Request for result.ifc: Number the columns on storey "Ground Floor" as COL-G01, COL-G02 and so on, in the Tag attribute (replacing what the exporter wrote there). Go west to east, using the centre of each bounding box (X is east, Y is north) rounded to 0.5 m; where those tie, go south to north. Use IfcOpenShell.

First a look at what the model holds.

```python
import ifcopenshell
import ifcopenshell.util.element
import ifcopenshell.util.placement

model = ifcopenshell.open("result.ifc")
print(model.schema)
storey = next(s for s in model.by_type("IfcBuildingStorey") if s.Name == "Ground Floor")
columns = [e for e in ifcopenshell.util.element.get_decomposition(storey) if e.is_a("IfcColumn")]
for e in sorted(columns, key=lambda e: e.id()):
    origin = ifcopenshell.util.placement.get_local_placement(e.ObjectPlacement)[:3, 3]
    print(e.id(), e.Tag, e.Name, origin.round(2) + 0.0, sep=" | ")
```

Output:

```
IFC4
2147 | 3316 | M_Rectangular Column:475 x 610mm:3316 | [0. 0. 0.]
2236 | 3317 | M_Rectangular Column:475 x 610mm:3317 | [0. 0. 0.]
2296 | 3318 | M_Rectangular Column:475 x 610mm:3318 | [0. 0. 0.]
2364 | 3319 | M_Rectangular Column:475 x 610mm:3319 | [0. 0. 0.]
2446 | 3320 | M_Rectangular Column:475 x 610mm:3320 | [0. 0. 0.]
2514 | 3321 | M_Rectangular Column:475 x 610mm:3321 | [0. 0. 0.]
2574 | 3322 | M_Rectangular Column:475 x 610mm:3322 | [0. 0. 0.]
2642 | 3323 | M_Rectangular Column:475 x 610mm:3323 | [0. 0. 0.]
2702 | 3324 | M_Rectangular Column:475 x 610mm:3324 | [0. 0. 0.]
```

```python
import ifcopenshell
import ifcopenshell.geom
import ifcopenshell.util.element
import ifcopenshell.util.shape

model = ifcopenshell.open("result.ifc")
settings = ifcopenshell.geom.settings()
settings.set("use-world-coords", True)


def centre(element):
    shape = ifcopenshell.geom.create_shape(settings, element)
    return ifcopenshell.util.shape.get_bbox_centroid(shape.geometry)


storey = next(s for s in model.by_type("IfcBuildingStorey") if s.Name == "Ground Floor")
columns = [e for e in ifcopenshell.util.element.get_decomposition(storey) if e.is_a("IfcColumn")]

# Insertion points can sit at a corner or the storey origin, so sort by the geometry (in metres).
centres = {e: centre(e) for e in columns}
columns.sort(key=lambda e: (round(centres[e][0] / 0.5), centres[e][1]))

for i, e in enumerate(columns, start=1):
    number = f"COL-G{i:02d}"
    e.Tag = number
    print(e.id(), number)

model.write("result-out.ifc")
```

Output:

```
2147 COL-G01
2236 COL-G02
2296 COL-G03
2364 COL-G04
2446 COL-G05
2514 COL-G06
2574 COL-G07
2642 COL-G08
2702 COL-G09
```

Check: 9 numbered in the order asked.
